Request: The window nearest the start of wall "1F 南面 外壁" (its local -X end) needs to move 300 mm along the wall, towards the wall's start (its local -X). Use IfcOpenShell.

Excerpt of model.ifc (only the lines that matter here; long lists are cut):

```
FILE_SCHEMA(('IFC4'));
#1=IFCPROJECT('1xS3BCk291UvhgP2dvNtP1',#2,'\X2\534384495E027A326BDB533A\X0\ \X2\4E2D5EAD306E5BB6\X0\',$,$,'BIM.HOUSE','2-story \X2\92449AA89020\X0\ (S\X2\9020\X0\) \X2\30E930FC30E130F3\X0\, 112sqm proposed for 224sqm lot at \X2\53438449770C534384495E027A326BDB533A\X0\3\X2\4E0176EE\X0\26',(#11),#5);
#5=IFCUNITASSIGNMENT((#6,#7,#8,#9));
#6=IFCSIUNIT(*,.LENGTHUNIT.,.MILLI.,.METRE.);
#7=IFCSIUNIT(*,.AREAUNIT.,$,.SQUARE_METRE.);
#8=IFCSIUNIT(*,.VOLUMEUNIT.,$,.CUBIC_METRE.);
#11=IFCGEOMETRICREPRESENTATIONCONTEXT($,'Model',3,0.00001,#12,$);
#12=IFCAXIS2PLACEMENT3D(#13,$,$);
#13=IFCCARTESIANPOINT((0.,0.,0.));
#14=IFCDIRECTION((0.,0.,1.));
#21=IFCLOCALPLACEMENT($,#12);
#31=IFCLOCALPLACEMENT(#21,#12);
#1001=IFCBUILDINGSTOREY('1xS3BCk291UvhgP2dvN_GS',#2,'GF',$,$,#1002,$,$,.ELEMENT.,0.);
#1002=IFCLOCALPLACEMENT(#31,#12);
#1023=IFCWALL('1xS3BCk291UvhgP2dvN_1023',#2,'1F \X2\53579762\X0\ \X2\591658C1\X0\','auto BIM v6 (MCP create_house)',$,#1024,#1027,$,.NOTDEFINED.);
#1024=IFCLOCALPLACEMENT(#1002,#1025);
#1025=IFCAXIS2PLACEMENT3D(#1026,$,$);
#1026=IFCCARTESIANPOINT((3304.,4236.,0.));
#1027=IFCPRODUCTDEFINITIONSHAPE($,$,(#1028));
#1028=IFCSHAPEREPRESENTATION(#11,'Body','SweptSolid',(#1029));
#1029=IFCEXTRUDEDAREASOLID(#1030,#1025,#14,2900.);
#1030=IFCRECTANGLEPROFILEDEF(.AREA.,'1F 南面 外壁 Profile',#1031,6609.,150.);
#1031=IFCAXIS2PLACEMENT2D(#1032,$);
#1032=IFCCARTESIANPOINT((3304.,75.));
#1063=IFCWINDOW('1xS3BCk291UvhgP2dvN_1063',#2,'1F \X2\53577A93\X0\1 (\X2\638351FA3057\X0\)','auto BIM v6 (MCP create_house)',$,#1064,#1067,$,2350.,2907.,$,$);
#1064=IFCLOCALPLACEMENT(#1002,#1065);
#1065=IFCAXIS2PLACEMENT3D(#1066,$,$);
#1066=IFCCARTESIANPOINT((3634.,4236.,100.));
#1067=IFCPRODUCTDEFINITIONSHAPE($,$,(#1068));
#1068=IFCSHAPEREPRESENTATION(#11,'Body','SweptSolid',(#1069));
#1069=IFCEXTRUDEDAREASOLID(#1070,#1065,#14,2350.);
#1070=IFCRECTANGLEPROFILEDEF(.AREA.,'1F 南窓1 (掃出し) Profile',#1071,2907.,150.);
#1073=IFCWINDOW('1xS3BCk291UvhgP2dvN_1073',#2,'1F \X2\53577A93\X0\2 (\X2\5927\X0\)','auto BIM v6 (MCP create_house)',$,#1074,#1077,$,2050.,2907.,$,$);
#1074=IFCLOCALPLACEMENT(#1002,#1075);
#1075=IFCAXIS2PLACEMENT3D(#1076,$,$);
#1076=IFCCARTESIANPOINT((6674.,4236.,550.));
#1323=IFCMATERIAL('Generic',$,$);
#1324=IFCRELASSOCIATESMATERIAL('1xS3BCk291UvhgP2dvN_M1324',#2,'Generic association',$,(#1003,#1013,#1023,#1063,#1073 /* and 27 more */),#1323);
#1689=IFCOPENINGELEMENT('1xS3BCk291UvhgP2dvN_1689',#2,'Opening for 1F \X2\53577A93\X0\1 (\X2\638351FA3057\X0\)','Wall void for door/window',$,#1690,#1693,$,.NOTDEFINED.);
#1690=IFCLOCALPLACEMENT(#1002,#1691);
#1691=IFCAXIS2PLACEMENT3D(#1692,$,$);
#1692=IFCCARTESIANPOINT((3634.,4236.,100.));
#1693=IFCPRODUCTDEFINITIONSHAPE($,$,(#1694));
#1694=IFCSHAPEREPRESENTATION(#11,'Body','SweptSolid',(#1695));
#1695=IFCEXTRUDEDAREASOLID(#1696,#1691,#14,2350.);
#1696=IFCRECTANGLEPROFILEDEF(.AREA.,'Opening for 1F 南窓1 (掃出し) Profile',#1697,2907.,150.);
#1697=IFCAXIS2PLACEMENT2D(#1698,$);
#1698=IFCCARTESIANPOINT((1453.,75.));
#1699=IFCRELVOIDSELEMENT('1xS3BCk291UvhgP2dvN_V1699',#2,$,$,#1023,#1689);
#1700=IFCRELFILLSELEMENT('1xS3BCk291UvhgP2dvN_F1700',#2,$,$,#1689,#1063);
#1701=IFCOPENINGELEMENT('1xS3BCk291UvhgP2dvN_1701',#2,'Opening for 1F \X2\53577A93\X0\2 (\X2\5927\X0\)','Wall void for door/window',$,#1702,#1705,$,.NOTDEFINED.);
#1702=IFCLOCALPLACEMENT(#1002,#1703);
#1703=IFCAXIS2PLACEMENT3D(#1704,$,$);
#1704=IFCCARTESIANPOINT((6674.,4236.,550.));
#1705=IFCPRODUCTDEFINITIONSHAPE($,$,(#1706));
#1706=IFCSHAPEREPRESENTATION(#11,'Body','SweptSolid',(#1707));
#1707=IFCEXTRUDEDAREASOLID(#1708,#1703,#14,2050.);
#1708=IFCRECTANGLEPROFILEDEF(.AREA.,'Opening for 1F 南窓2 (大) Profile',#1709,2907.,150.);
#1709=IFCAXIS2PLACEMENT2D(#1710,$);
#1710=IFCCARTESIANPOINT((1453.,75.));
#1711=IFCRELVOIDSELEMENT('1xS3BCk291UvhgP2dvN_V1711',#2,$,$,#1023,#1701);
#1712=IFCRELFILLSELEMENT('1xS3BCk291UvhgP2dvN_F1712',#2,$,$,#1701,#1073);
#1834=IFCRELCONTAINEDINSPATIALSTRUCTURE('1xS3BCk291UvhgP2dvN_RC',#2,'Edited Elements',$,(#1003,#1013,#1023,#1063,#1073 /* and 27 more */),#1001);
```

```python
import ifcopenshell
import ifcopenshell.api.geometry
import ifcopenshell.util.placement
import ifcopenshell.util.unit

model = ifcopenshell.open("model.ifc")
unit_scale = ifcopenshell.util.unit.calculate_unit_scale(model)

window = model.by_guid("1xS3BCk291UvhgP2dvN_1063")
opening = window.FillsVoids[0].RelatingOpeningElement
wall = opening.VoidsElements[0].RelatingBuildingElement

wall_matrix = ifcopenshell.util.placement.get_local_placement(wall.ObjectPlacement)
shift = wall_matrix[:3, 0] * -0.3 / unit_scale
before = ifcopenshell.util.placement.get_local_placement(window.ObjectPlacement)[:3, 3].copy()

# The window is not placed relative to its opening, so move both.
for product in (opening, window):
    matrix = ifcopenshell.util.placement.get_local_placement(product.ObjectPlacement)
    matrix[:3, 3] += shift
    ifcopenshell.api.geometry.edit_object_placement(model, product=product, matrix=matrix, is_si=False)

after = ifcopenshell.util.placement.get_local_placement(window.ObjectPlacement)[:3, 3]
print("window moved by", (after - before).round(3) + 0.0)

model.write("model_updated.ifc")
```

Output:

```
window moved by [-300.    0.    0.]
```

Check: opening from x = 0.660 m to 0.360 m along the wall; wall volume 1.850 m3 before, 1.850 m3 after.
